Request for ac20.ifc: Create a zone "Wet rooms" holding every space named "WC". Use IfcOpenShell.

First a look at what the model holds.

```python
import ifcopenshell

model = ifcopenshell.open("ac20.ifc")
print(model.schema)
seen = {}
for space in model.by_type("IfcSpace"):
    seen[space.LongName] = seen.get(space.LongName, 0) + 1
for name, count in sorted(seen.items(), key=str):
    print(count, "x", name)
print("zones:", [z.Name for z in model.by_type("IfcZone")][:20])
```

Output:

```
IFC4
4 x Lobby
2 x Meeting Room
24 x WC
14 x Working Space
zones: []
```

```python
import ifcopenshell
import ifcopenshell.api.group
import ifcopenshell.api.root

model = ifcopenshell.open("ac20.ifc")

names = {"WC"}
spaces = [s for s in model.by_type("IfcSpace") if s.LongName in names]

zone = ifcopenshell.api.root.create_entity(model, ifc_class="IfcZone", name="Wet rooms")
ifcopenshell.api.group.assign_group(model, products=spaces, group=zone)
print(len(spaces), "spaces in", zone.Name)

model.write("ac20-out.ifc")
```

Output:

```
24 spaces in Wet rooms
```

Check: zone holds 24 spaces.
